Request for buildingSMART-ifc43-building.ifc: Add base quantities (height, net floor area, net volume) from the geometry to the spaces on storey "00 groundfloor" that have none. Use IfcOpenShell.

First a look at what the model holds.

```python
import ifcopenshell
import ifcopenshell.util.element
import ifcopenshell.util.unit

model = ifcopenshell.open("buildingSMART-ifc43-building.ifc")
print(model.schema)
for unit_type in ("LENGTHUNIT", "AREAUNIT", "VOLUMEUNIT"):
    print(unit_type, ifcopenshell.util.unit.calculate_unit_scale(model, unit_type))
storey = next(s for s in model.by_type("IfcBuildingStorey") if s.Name == "00 groundfloor")
spaces = [e for e in ifcopenshell.util.element.get_decomposition(storey) if e.is_a("IfcSpace")]
for e in sorted(spaces, key=lambda e: e.id()):
    print(e.id(), e.is_a(), e.Name, list(ifcopenshell.util.element.get_psets(e, qtos_only=True)), sep=" | ")
```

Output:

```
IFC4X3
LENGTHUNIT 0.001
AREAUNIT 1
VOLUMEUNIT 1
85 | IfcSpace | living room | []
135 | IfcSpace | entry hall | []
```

```python
import ifcopenshell
import ifcopenshell.api.pset
import ifcopenshell.geom
import ifcopenshell.util.element
import ifcopenshell.util.shape
import ifcopenshell.util.unit

model = ifcopenshell.open("buildingSMART-ifc43-building.ifc")
unit_scale = ifcopenshell.util.unit.calculate_unit_scale(model)
area_scale = ifcopenshell.util.unit.calculate_unit_scale(model, "AREAUNIT")
volume_scale = ifcopenshell.util.unit.calculate_unit_scale(model, "VOLUMEUNIT")
settings = ifcopenshell.geom.settings()

storey = next(s for s in model.by_type("IfcBuildingStorey") if s.Name == "00 groundfloor")
spaces = [e for e in ifcopenshell.util.element.get_decomposition(storey) if e.is_a("IfcSpace")]

for e in sorted(spaces, key=lambda e: e.id()):
    if ifcopenshell.util.element.get_psets(e, qtos_only=True, should_inherit=False):
        continue
    # Geometry comes back in metres, in the element's own axes.
    shape = ifcopenshell.geom.create_shape(settings, e)
    values = {
        "Height": ifcopenshell.util.shape.get_z(shape.geometry) / unit_scale,
        "NetFloorArea": ifcopenshell.util.shape.get_footprint_area(shape.geometry) / area_scale,
        "NetVolume": ifcopenshell.util.shape.get_volume(shape.geometry) / volume_scale,
    }
    qto = ifcopenshell.api.pset.add_qto(model, product=e, name="Qto_SpaceBaseQuantities")
    ifcopenshell.api.pset.edit_qto(model, qto=qto, properties=values)
    print(e.id(), {k: round(v, 3) for k, v in values.items()})

model.write("buildingSMART-ifc43-building_updated.ifc")
```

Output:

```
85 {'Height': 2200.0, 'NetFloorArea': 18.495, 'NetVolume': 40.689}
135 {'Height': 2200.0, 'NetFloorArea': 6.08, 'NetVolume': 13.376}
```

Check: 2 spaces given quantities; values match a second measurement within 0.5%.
